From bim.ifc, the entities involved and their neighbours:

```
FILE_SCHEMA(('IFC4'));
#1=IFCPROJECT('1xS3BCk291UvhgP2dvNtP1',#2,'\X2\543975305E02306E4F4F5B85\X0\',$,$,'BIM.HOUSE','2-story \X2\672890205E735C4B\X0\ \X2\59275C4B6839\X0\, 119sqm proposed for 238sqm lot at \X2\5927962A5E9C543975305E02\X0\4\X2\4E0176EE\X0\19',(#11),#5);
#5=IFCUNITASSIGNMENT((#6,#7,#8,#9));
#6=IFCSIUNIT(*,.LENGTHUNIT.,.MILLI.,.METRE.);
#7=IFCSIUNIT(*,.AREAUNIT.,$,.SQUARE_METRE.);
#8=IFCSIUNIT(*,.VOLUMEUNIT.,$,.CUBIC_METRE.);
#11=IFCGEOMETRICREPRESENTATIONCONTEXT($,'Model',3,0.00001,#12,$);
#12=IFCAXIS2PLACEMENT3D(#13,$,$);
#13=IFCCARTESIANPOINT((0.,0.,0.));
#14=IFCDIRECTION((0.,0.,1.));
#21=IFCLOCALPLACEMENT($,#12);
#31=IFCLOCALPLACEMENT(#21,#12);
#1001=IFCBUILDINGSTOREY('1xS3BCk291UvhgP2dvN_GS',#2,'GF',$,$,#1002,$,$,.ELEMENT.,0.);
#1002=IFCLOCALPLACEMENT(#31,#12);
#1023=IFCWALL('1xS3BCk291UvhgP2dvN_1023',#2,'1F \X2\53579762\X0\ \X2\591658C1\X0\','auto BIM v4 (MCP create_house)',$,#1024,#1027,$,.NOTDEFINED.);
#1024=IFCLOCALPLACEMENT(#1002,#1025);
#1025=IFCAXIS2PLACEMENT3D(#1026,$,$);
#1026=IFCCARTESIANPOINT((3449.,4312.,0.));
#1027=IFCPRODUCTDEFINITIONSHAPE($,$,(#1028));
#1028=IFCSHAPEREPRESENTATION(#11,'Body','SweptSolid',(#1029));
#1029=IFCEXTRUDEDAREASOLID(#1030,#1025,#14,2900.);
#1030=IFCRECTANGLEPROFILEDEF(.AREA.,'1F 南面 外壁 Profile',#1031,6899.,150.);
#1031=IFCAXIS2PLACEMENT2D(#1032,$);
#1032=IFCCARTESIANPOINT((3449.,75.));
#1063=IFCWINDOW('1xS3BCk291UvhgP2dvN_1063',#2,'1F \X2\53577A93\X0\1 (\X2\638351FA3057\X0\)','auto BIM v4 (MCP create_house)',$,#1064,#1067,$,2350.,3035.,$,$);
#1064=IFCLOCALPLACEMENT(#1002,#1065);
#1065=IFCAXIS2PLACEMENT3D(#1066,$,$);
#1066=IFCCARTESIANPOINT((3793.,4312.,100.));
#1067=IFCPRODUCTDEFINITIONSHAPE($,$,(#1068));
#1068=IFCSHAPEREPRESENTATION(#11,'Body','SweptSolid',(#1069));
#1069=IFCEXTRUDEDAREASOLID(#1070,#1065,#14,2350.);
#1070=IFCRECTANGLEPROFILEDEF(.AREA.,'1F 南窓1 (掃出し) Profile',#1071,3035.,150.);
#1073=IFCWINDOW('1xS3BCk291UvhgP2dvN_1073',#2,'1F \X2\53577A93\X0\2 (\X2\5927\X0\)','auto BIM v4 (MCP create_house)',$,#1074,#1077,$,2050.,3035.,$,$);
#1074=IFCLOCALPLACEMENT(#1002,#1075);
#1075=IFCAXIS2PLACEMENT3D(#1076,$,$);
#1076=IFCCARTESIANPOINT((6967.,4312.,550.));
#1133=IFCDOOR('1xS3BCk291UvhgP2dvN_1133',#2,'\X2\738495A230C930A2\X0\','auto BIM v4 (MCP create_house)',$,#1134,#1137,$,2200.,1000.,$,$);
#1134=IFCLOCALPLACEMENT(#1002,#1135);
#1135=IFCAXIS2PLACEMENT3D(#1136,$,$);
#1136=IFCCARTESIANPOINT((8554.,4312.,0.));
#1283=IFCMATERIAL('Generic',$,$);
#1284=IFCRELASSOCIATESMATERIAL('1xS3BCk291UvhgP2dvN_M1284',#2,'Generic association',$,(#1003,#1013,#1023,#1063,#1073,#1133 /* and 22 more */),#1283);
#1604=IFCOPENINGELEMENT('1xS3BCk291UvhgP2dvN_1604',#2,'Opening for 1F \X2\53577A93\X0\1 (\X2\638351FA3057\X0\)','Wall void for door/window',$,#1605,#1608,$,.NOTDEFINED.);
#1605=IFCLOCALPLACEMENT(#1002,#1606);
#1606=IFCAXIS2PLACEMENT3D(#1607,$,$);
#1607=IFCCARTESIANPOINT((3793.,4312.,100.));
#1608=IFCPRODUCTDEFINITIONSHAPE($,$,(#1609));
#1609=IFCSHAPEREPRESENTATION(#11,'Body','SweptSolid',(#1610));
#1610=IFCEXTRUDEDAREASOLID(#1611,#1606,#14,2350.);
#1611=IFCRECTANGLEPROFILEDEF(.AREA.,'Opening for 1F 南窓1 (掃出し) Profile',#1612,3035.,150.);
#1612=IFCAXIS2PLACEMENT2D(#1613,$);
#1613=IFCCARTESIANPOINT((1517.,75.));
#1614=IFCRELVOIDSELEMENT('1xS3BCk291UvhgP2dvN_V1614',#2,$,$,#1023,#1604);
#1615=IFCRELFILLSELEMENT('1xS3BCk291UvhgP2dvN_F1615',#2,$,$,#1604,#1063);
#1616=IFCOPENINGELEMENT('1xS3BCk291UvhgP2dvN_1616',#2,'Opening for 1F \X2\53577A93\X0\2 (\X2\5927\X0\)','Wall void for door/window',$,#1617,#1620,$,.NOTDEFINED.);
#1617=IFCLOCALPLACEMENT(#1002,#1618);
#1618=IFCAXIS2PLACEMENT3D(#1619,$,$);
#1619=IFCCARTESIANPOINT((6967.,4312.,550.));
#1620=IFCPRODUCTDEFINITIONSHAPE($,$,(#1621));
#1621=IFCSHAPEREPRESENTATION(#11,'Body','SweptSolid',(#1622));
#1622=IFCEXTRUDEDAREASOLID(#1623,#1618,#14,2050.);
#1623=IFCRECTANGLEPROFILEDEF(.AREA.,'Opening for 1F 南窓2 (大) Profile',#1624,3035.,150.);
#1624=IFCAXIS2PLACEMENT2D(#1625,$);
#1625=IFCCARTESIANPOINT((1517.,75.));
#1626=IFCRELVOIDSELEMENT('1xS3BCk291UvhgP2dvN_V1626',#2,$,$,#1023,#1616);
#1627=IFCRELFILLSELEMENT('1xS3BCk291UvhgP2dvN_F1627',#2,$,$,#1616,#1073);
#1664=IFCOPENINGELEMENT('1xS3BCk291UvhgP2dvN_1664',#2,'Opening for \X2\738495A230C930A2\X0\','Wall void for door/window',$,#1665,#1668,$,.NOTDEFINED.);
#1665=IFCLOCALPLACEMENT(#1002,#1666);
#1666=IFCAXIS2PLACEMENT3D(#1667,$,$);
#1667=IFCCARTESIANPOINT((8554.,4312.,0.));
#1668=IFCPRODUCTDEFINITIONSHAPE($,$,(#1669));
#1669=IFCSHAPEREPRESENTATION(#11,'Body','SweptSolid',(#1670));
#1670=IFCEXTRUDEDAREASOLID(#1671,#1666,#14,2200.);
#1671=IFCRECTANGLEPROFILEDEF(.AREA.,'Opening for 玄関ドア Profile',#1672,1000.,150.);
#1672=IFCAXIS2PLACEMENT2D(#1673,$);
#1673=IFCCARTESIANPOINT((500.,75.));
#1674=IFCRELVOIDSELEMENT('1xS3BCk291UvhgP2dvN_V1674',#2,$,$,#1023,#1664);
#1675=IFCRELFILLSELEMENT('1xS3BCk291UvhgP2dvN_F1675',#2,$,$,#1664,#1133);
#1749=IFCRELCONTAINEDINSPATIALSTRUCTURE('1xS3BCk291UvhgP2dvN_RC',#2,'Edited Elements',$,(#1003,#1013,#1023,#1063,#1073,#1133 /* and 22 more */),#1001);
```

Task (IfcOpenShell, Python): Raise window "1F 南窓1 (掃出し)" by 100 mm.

```python
import numpy as np
import ifcopenshell
import ifcopenshell.api.geometry
import ifcopenshell.util.placement
import ifcopenshell.util.unit

model = ifcopenshell.open("bim.ifc")
unit_scale = ifcopenshell.util.unit.calculate_unit_scale(model)

window = model.by_id(1063)
opening = window.FillsVoids[0].RelatingOpeningElement
dz = 0.1 / unit_scale

shift = np.array([0.0, 0.0, dz])
# The window is not placed relative to its opening, so move both.
for product in (opening, window):
    matrix = ifcopenshell.util.placement.get_local_placement(product.ObjectPlacement)
    matrix[:3, 3] += shift
    ifcopenshell.api.geometry.edit_object_placement(model, product=product, matrix=matrix, is_si=False)

print(f"moved by {dz * unit_scale:+.3f} m")

model.write("bim_updated.ifc")
```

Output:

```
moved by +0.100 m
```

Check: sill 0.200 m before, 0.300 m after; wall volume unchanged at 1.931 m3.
